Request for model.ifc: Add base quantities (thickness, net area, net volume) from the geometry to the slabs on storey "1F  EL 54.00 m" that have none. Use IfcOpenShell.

First a look at what the model holds.

```python
import ifcopenshell
import ifcopenshell.util.element
import ifcopenshell.util.unit

model = ifcopenshell.open("model.ifc")
print(model.schema)
for unit_type in ("LENGTHUNIT", "AREAUNIT", "VOLUMEUNIT"):
    print(unit_type, ifcopenshell.util.unit.calculate_unit_scale(model, unit_type))
storey = next(s for s in model.by_type("IfcBuildingStorey") if s.Name == "1F  EL 54.00 m")
slabs = [e for e in ifcopenshell.util.element.get_decomposition(storey) if e.is_a("IfcSlab")]
for e in sorted(slabs, key=lambda e: e.id()):
    print(e.id(), e.is_a(), e.Name, list(ifcopenshell.util.element.get_psets(e, qtos_only=True)), sep=" | ")
```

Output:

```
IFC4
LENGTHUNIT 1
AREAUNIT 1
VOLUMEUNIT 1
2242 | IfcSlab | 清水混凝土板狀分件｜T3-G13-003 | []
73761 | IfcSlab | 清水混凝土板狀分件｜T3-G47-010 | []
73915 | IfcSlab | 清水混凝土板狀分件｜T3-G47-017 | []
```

```python
import ifcopenshell
import ifcopenshell.api.pset
import ifcopenshell.geom
import ifcopenshell.util.element
import ifcopenshell.util.shape
import ifcopenshell.util.unit

model = ifcopenshell.open("model.ifc")
unit_scale = ifcopenshell.util.unit.calculate_unit_scale(model)
area_scale = ifcopenshell.util.unit.calculate_unit_scale(model, "AREAUNIT")
volume_scale = ifcopenshell.util.unit.calculate_unit_scale(model, "VOLUMEUNIT")
settings = ifcopenshell.geom.settings()

storey = next(s for s in model.by_type("IfcBuildingStorey") if s.Name == "1F  EL 54.00 m")
slabs = [e for e in ifcopenshell.util.element.get_decomposition(storey) if e.is_a("IfcSlab")]

for e in sorted(slabs, key=lambda e: e.id()):
    if ifcopenshell.util.element.get_psets(e, qtos_only=True, should_inherit=False):
        continue
    # Geometry comes back in metres, in the element's own axes.
    shape = ifcopenshell.geom.create_shape(settings, e)
    values = {
        "Width": ifcopenshell.util.shape.get_z(shape.geometry) / unit_scale,
        "NetArea": ifcopenshell.util.shape.get_footprint_area(shape.geometry) / area_scale,
        "NetVolume": ifcopenshell.util.shape.get_volume(shape.geometry) / volume_scale,
    }
    qto = ifcopenshell.api.pset.add_qto(model, product=e, name="Qto_SlabBaseQuantities")
    ifcopenshell.api.pset.edit_qto(model, qto=qto, properties=values)
    print(e.id(), {k: round(v, 3) for k, v in values.items()})

model.write("model_edited.ifc")
```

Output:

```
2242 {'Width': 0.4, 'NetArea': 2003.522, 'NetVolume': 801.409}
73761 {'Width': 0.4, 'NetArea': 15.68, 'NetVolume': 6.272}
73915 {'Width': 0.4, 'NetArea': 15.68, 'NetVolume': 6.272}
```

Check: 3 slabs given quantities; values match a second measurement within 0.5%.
